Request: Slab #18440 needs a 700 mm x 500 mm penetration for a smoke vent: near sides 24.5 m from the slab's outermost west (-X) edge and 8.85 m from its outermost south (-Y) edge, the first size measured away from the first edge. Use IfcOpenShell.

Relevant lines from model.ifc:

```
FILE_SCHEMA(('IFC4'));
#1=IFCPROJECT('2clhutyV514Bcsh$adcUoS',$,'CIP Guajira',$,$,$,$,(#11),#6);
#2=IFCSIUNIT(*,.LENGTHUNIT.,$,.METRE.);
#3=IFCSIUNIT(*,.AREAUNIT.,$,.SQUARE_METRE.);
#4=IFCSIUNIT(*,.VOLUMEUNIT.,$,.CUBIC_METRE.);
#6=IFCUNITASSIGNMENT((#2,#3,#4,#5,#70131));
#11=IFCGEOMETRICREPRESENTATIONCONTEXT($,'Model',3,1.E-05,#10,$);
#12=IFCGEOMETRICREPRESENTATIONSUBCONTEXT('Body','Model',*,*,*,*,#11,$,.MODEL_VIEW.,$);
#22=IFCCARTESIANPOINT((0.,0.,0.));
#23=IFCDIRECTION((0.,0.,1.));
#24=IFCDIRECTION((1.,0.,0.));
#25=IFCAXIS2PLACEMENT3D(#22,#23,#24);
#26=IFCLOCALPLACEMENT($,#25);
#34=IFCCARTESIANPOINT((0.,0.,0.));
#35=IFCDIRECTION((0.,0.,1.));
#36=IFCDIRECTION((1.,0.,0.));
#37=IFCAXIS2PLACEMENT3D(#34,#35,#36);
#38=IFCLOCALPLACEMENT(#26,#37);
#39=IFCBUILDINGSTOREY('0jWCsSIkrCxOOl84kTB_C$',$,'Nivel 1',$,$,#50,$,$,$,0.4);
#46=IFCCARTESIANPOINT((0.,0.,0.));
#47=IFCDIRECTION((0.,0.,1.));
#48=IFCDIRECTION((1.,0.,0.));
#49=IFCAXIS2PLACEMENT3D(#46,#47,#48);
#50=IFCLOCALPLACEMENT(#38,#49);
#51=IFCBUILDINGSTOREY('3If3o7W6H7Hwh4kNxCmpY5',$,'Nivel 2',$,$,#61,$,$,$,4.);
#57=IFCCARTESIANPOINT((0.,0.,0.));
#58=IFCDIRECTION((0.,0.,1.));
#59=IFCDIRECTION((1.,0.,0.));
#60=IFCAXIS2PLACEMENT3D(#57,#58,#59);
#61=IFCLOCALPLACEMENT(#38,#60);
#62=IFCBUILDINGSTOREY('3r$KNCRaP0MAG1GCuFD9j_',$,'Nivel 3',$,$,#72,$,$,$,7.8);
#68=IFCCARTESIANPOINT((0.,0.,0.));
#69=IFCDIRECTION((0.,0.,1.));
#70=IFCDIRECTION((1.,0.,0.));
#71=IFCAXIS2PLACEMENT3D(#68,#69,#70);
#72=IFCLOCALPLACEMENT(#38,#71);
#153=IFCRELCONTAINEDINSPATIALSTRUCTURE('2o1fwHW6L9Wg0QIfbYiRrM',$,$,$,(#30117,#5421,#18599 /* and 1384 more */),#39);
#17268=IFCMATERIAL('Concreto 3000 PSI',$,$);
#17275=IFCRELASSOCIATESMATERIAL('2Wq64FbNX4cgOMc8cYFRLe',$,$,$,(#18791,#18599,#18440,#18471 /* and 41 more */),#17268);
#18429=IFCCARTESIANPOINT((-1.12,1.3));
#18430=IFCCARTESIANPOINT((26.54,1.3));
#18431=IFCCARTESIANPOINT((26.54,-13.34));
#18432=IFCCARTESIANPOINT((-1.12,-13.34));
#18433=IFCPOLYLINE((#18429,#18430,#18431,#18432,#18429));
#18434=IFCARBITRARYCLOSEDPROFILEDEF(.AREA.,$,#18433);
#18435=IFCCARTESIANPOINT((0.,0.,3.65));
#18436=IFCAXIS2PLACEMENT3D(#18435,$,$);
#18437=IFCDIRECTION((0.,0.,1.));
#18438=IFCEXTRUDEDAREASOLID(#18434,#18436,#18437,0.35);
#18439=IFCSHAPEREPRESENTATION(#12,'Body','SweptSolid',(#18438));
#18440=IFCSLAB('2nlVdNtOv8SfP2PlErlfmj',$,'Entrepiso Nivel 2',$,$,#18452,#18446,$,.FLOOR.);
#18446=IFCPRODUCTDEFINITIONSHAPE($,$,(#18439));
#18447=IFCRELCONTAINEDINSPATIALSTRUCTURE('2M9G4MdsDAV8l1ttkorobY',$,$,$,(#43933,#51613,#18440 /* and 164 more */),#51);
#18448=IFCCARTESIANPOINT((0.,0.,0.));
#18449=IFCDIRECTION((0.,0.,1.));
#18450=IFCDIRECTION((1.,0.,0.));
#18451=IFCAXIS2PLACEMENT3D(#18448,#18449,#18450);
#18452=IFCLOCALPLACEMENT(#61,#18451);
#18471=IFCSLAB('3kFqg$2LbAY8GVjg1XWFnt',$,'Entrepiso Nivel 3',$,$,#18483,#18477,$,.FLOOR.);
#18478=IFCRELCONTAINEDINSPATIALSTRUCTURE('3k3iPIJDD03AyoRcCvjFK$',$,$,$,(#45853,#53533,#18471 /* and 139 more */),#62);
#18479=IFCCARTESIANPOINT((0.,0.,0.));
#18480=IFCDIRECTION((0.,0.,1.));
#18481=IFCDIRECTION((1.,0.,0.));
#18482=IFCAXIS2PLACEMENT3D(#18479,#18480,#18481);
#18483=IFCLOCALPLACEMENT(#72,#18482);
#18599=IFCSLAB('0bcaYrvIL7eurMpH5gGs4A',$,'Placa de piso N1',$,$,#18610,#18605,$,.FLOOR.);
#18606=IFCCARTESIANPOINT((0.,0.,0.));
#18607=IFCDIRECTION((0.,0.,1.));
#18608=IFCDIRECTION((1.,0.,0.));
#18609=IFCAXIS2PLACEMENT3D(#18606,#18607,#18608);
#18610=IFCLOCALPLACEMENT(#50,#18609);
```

```python
import numpy as np
import ifcopenshell
import ifcopenshell.api.feature
import ifcopenshell.api.geometry
import ifcopenshell.api.root
import ifcopenshell.geom
import ifcopenshell.util.placement
import ifcopenshell.util.representation
import ifcopenshell.util.shape
import ifcopenshell.util.unit

model = ifcopenshell.open("model.ifc")
unit_scale = ifcopenshell.util.unit.calculate_unit_scale(model)
settings = ifcopenshell.geom.settings()


def volume(element):
    """Net volume in cubic metres, openings subtracted."""
    shape = ifcopenshell.geom.create_shape(settings, element)
    return ifcopenshell.util.shape.get_volume(shape.geometry)


slab = model.by_guid("2nlVdNtOv8SfP2PlErlfmj")
before = volume(slab)

# Extent in the slab's own axes, in metres. The edges named are its -X and -Y sides.
slab_shape = ifcopenshell.geom.create_shape(settings, slab)
vertices = ifcopenshell.util.shape.get_vertices(slab_shape.geometry)
x_min, y_min, bottom = vertices.min(axis=0)
top = vertices[:, 2].max()

opening = ifcopenshell.api.root.create_entity(model, ifc_class="IfcOpeningElement", name="Smoke vent opening", predefined_type="OPENING")
context = ifcopenshell.util.representation.get_context(model, "Model", "Body", "MODEL_VIEW")
width, depth = 0.7, 0.5
outline = [(0.0, 0.0), (width, 0.0), (width, depth), (0.0, depth), (0.0, 0.0)]
# Overshoot both faces by 50 mm so the cut is clean.
shape = ifcopenshell.api.geometry.add_slab_representation(
    model, context=context, depth=top - bottom + 0.1, polyline=outline
)
ifcopenshell.api.geometry.assign_representation(model, product=opening, representation=shape)

matrix = ifcopenshell.util.placement.get_local_placement(slab.ObjectPlacement)
matrix[:, 3] = matrix @ np.append(np.array([x_min + 24.5, y_min + 8.85, bottom - 0.05]) / unit_scale, 1.0)
ifcopenshell.api.geometry.edit_object_placement(model, product=opening, matrix=matrix, is_si=False)
ifcopenshell.api.feature.add_feature(model, feature=opening, element=slab)

after = volume(slab)

print(f"slab volume {before:.3f} -> {after:.3f} m3")

model.write("model_rev.ifc")
```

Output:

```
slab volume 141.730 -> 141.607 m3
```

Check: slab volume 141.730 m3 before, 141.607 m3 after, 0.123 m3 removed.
